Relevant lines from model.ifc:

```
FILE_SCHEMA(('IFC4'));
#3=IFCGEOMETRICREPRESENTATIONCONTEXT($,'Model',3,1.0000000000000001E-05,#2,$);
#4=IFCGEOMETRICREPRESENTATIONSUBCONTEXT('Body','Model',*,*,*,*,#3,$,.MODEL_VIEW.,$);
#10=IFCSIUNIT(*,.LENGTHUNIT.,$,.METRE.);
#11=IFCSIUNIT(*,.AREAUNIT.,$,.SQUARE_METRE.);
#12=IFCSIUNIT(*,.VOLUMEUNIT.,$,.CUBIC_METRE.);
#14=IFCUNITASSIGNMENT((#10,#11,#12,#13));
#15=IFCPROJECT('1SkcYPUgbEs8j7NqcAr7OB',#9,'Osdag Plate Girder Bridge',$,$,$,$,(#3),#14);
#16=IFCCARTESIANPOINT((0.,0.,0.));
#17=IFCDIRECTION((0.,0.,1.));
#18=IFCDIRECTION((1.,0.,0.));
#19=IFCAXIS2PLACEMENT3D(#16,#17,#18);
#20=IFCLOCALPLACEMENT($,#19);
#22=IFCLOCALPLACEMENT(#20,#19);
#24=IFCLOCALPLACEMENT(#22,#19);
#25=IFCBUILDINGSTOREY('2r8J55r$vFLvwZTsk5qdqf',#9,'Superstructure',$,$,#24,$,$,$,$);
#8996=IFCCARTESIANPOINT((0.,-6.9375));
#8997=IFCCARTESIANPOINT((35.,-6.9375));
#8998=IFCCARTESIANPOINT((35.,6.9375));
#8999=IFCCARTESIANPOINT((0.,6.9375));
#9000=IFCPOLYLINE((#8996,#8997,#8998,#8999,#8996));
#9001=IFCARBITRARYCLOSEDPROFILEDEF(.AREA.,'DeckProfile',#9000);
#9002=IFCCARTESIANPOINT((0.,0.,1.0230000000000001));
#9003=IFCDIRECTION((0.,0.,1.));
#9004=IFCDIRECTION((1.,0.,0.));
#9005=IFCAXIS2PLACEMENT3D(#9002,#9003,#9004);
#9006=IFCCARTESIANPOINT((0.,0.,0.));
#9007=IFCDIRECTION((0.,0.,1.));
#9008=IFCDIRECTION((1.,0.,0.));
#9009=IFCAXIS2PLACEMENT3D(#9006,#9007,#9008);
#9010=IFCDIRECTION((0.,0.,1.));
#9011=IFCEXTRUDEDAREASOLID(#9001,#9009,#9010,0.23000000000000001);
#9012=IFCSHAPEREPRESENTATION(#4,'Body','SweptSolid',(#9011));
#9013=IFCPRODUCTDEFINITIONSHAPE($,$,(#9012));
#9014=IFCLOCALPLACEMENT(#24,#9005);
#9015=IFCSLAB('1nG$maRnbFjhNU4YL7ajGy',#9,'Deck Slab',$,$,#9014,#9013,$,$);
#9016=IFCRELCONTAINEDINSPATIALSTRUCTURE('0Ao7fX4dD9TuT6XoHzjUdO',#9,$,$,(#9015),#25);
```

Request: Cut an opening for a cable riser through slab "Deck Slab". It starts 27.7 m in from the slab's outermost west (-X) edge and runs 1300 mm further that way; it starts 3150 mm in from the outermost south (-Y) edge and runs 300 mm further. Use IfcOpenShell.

```python
import numpy as np
import ifcopenshell
import ifcopenshell.api.feature
import ifcopenshell.api.geometry
import ifcopenshell.api.root
import ifcopenshell.geom
import ifcopenshell.util.placement
import ifcopenshell.util.representation
import ifcopenshell.util.shape
import ifcopenshell.util.unit

model = ifcopenshell.open("model.ifc")
unit_scale = ifcopenshell.util.unit.calculate_unit_scale(model)
settings = ifcopenshell.geom.settings()


def volume(element):
    """Net volume in cubic metres, openings subtracted."""
    shape = ifcopenshell.geom.create_shape(settings, element)
    return ifcopenshell.util.shape.get_volume(shape.geometry)


slab = model.by_id(9015)
before = volume(slab)

# Extent in the slab's own axes, in metres. The edges named are its -X and -Y sides.
slab_shape = ifcopenshell.geom.create_shape(settings, slab)
vertices = ifcopenshell.util.shape.get_vertices(slab_shape.geometry)
x_min, y_min, bottom = vertices.min(axis=0)
top = vertices[:, 2].max()

opening = ifcopenshell.api.root.create_entity(model, ifc_class="IfcOpeningElement", name="Cable riser opening", predefined_type="OPENING")
context = ifcopenshell.util.representation.get_context(model, "Model", "Body", "MODEL_VIEW")
width, depth = 1.3, 0.3
outline = [(0.0, 0.0), (width, 0.0), (width, depth), (0.0, depth), (0.0, 0.0)]
# Overshoot both faces by 50 mm so the cut is clean.
shape = ifcopenshell.api.geometry.add_slab_representation(
    model, context=context, depth=top - bottom + 0.1, polyline=outline
)
ifcopenshell.api.geometry.assign_representation(model, product=opening, representation=shape)

matrix = ifcopenshell.util.placement.get_local_placement(slab.ObjectPlacement)
matrix[:, 3] = matrix @ np.append(np.array([x_min + 27.7, y_min + 3.15, bottom - 0.05]) / unit_scale, 1.0)
ifcopenshell.api.geometry.edit_object_placement(model, product=opening, matrix=matrix, is_si=False)
ifcopenshell.api.feature.add_feature(model, feature=opening, element=slab)

after = volume(slab)

print(f"slab volume {before:.3f} -> {after:.3f} m3")

model.write("model_edited.ifc")
```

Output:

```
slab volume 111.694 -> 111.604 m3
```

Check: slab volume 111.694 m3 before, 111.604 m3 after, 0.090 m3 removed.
